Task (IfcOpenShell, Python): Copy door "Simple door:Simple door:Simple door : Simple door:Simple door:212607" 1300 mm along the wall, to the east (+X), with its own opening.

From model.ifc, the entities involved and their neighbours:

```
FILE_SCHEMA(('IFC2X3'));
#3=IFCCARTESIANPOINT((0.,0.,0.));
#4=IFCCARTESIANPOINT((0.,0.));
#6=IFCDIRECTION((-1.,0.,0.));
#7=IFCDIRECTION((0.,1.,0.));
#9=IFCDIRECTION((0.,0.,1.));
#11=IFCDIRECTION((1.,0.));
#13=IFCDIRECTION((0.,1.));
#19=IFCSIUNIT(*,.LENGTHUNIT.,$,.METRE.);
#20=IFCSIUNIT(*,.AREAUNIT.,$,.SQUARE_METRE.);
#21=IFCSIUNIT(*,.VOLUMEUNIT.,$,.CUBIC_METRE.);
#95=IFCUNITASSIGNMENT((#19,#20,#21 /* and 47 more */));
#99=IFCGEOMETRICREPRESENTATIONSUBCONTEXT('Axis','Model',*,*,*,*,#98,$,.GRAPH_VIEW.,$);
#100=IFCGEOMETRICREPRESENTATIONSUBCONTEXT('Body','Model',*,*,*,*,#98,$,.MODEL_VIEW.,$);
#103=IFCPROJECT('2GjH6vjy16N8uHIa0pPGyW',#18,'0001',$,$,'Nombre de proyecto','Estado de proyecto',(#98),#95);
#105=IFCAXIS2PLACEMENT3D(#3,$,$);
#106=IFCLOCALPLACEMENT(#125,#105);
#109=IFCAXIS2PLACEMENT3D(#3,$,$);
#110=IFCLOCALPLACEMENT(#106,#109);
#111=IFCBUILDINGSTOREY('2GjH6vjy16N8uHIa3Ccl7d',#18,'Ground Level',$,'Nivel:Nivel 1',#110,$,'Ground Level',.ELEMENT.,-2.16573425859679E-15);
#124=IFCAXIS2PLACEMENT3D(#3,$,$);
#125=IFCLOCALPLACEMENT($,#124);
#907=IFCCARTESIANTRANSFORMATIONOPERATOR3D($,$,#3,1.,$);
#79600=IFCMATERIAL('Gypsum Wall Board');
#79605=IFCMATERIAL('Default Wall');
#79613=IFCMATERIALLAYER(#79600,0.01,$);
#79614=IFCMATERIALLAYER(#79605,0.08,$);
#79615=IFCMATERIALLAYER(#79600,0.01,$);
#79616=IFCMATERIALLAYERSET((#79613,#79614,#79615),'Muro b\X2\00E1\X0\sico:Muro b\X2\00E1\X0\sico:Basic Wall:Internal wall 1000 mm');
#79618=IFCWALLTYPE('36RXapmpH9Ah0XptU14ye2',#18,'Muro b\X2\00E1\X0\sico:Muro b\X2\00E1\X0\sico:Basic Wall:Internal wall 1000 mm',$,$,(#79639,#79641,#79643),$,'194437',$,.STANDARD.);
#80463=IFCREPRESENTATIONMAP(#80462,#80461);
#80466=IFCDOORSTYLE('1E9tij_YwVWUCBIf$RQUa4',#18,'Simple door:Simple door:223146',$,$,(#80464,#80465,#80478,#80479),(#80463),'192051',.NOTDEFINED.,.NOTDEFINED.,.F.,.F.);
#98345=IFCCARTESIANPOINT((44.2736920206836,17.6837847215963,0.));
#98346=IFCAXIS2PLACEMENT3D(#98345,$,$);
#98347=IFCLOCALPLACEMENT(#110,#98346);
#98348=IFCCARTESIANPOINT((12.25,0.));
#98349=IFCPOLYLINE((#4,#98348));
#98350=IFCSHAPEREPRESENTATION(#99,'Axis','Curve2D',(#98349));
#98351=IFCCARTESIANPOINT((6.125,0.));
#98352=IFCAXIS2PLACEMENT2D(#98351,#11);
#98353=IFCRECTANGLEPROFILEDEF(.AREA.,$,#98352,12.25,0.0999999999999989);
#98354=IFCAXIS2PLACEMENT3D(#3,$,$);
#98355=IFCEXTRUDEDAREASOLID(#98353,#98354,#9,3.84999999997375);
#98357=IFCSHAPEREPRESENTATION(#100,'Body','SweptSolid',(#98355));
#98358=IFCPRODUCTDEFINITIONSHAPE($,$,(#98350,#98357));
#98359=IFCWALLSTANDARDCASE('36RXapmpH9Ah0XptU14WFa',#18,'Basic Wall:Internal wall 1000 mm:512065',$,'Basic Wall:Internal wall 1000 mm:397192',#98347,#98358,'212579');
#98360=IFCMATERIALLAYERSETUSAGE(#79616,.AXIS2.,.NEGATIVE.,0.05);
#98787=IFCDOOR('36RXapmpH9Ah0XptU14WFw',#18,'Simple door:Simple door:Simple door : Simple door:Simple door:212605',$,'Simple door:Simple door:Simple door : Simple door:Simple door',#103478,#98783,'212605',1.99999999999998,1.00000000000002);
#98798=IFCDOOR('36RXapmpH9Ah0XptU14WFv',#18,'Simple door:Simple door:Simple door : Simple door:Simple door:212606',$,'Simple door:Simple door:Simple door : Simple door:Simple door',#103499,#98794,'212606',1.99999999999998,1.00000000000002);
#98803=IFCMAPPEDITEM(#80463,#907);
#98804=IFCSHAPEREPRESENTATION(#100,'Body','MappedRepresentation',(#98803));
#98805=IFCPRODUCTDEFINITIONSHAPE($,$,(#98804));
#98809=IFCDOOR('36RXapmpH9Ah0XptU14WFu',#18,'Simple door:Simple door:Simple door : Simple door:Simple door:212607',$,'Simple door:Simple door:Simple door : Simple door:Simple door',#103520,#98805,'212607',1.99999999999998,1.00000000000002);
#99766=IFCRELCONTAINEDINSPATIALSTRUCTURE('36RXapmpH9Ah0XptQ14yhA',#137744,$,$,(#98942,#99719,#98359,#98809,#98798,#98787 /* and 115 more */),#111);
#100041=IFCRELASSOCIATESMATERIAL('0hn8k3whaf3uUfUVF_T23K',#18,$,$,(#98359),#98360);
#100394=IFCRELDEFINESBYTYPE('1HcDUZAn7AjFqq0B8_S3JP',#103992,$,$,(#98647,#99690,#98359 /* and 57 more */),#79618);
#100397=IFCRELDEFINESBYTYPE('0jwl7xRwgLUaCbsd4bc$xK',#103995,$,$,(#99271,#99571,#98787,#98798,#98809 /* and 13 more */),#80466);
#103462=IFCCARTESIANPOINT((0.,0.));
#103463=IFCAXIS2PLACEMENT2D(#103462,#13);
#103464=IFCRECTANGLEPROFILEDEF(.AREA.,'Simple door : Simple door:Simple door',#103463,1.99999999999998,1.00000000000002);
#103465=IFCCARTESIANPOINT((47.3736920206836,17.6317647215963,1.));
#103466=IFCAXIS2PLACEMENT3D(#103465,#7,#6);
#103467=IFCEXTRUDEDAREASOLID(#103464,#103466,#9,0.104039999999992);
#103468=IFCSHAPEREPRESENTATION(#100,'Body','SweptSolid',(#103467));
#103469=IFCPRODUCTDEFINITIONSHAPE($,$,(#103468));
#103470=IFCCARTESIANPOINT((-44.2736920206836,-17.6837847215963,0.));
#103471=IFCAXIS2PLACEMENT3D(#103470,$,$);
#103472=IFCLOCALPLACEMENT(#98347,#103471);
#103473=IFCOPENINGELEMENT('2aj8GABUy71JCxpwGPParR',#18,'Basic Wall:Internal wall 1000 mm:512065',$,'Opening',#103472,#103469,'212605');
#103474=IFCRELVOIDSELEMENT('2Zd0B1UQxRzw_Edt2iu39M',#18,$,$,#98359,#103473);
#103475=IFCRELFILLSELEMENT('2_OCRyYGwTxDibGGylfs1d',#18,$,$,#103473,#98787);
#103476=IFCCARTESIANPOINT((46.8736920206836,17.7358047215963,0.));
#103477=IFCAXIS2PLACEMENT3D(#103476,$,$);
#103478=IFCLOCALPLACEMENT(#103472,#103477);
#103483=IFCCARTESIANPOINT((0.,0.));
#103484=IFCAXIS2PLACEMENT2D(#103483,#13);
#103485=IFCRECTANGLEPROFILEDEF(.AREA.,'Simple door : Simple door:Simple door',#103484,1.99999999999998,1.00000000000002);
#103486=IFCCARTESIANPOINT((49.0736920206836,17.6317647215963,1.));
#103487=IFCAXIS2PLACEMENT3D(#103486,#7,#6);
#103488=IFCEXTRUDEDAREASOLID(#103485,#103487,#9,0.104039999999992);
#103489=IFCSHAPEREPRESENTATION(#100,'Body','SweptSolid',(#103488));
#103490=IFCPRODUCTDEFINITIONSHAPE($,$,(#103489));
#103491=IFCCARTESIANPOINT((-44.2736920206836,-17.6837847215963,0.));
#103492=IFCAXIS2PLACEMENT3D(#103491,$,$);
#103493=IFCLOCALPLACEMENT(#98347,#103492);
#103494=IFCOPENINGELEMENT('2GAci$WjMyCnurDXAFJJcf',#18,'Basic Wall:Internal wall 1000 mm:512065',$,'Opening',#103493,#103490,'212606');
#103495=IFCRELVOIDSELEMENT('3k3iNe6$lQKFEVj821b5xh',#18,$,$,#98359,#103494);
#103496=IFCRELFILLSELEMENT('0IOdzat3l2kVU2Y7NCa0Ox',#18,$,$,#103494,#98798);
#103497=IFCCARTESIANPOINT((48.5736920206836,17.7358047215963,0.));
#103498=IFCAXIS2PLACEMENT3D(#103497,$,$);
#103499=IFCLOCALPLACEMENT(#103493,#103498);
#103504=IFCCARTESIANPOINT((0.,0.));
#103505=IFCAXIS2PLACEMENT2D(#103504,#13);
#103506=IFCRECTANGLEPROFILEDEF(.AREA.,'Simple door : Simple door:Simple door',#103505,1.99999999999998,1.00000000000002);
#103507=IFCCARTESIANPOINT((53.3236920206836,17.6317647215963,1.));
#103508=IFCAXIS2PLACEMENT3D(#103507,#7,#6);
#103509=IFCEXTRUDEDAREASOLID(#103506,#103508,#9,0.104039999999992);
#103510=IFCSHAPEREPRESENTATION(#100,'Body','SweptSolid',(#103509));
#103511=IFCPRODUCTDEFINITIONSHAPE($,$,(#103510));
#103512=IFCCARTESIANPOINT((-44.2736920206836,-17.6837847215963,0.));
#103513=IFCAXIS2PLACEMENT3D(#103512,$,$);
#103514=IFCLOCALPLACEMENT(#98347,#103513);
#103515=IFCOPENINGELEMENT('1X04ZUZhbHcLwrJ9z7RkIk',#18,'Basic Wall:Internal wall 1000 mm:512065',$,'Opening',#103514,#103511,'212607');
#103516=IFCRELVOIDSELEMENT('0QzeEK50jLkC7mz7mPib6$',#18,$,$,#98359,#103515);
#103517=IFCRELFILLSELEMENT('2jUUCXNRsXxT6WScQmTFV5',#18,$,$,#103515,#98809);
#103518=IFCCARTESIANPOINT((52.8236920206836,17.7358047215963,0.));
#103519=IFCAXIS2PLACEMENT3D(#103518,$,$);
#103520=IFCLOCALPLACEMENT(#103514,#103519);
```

```python
import ifcopenshell
import ifcopenshell.api.feature
import ifcopenshell.api.geometry
import ifcopenshell.api.root
import ifcopenshell.geom
import ifcopenshell.util.element
import ifcopenshell.util.placement
import ifcopenshell.util.shape

model = ifcopenshell.open("model.ifc")
settings = ifcopenshell.geom.settings()


def volume(element):
    """Net volume in cubic metres, openings subtracted."""
    shape = ifcopenshell.geom.create_shape(settings, element)
    return ifcopenshell.util.shape.get_volume(shape.geometry)


def reuse_history(source, copy):
    """copy_class also copies each property set's owner history, people and application; keep the originals."""
    for rel in copy.IsDefinedBy:
        if rel.is_a("IfcRelDefinesByProperties") and (history := rel.RelatingPropertyDefinition.OwnerHistory):
            rel.RelatingPropertyDefinition.OwnerHistory = source.OwnerHistory
            ifcopenshell.util.element.remove_deep2(model, history)


door = model.by_guid("36RXapmpH9Ah0XptU14WFu")
opening = door.FillsVoids[0].RelatingOpeningElement
wall = opening.VoidsElements[0].RelatingBuildingElement
before = volume(wall)
shift = ifcopenshell.util.placement.get_local_placement(wall.ObjectPlacement)[:3, 0] * 1.3

# copy_class copies the void relationship, type, container and properties, but no geometry.
new_opening = ifcopenshell.api.root.copy_class(model, product=opening)
new_opening.Representation = ifcopenshell.util.element.copy_deep(
    model, opening.Representation, exclude=["IfcGeometricRepresentationContext", "IfcRepresentationMap"]
)
new_opening.Name = "Basic Wall:Internal wall 1000 mm"
new_opening.Tag = None
new_door = ifcopenshell.api.root.copy_class(model, product=door)
new_door.Representation = ifcopenshell.util.element.copy_deep(
    model, door.Representation, exclude=["IfcGeometricRepresentationContext", "IfcRepresentationMap"]
)
new_door.Name = "Simple door:Simple door:Simple door : Simple door:Simple door"
new_door.Tag = None
reuse_history(door, new_door)
fills = ifcopenshell.api.feature.add_filling(model, opening=new_opening, element=new_door)
fills.OwnerHistory = new_door.OwnerHistory  # required in IFC2X3

for old, new in ((opening, new_opening), (door, new_door)):
    matrix = ifcopenshell.util.placement.get_local_placement(old.ObjectPlacement)
    matrix[:3, 3] += shift
    ifcopenshell.api.geometry.edit_object_placement(model, product=new, matrix=matrix, is_si=False)

after = volume(wall)

print(f"wall volume {before:.3f} -> {after:.3f} m3")

model.write("model_updated.ifc")
```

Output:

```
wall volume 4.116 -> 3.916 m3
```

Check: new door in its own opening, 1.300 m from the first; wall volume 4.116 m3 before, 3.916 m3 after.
